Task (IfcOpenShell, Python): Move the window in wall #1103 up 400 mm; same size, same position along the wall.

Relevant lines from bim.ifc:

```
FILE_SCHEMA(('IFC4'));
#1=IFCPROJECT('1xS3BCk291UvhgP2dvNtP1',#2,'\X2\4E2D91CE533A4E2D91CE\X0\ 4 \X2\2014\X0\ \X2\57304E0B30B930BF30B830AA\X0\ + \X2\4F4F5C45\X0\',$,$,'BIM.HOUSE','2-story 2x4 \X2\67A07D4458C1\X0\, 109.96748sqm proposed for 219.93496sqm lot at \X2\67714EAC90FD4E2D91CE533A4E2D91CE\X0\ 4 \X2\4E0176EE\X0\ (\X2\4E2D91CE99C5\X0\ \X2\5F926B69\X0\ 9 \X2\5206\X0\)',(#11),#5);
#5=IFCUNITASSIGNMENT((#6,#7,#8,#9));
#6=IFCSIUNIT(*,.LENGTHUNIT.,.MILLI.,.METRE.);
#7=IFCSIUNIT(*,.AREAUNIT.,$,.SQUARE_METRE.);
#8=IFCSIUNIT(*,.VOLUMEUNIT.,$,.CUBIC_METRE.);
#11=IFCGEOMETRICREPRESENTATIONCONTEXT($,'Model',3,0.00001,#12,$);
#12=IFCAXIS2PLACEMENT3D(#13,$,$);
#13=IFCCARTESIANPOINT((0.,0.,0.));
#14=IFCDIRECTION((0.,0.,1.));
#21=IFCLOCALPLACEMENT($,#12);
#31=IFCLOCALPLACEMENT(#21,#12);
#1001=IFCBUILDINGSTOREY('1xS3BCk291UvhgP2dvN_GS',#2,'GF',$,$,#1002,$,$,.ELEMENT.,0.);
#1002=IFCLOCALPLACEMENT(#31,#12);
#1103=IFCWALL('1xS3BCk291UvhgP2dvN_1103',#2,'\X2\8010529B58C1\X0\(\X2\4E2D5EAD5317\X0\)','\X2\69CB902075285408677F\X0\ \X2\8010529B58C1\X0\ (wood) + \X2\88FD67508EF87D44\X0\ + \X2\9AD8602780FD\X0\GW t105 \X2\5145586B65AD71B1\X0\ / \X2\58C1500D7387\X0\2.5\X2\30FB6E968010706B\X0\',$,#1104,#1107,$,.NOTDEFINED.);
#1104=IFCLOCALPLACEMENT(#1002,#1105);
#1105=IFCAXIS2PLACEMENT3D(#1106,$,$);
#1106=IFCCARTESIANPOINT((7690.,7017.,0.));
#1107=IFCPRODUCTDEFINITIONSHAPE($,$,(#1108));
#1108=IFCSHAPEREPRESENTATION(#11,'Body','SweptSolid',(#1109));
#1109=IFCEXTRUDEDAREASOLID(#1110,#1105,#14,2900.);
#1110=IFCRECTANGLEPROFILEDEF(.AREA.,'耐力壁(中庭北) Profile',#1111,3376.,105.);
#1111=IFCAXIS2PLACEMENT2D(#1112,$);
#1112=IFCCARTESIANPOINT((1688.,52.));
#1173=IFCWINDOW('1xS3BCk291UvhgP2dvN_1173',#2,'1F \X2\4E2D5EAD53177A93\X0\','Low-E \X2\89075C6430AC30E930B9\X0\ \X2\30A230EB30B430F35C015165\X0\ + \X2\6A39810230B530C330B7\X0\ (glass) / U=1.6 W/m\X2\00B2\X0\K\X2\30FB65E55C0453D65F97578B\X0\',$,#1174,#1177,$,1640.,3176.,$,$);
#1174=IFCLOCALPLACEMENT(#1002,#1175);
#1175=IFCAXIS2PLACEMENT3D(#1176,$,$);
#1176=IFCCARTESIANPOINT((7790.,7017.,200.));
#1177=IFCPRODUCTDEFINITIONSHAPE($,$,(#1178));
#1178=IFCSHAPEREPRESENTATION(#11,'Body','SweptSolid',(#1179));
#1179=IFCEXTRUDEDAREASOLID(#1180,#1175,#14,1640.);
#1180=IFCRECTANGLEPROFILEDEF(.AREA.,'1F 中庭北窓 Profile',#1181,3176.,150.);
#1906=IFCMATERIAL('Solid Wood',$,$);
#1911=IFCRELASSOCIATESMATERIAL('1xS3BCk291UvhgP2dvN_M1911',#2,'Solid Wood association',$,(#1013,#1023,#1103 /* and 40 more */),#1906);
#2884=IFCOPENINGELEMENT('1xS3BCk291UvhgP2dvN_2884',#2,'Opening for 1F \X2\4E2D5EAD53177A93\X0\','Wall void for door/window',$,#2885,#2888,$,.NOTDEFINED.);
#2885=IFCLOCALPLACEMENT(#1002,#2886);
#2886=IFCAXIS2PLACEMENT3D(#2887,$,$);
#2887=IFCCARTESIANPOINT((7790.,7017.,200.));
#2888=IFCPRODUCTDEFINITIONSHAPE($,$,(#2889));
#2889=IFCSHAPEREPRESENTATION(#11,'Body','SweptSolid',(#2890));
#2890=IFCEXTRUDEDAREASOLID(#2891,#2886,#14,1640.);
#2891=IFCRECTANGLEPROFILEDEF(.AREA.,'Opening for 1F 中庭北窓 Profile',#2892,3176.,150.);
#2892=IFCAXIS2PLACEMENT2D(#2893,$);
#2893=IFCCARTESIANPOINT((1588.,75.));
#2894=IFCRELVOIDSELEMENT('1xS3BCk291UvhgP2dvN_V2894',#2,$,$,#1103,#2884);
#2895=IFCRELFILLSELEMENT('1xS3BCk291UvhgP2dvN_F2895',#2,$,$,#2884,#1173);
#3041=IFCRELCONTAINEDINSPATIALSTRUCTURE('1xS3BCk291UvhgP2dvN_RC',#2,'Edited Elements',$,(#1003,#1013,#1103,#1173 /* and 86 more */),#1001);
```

```python
import numpy as np
import ifcopenshell
import ifcopenshell.api.geometry
import ifcopenshell.util.placement
import ifcopenshell.util.unit

model = ifcopenshell.open("bim.ifc")
unit_scale = ifcopenshell.util.unit.calculate_unit_scale(model)

window = model.by_id(1173)
opening = window.FillsVoids[0].RelatingOpeningElement
dz = 0.4 / unit_scale

shift = np.array([0.0, 0.0, dz])
# The window is not placed relative to its opening, so move both.
for product in (opening, window):
    matrix = ifcopenshell.util.placement.get_local_placement(product.ObjectPlacement)
    matrix[:3, 3] += shift
    ifcopenshell.api.geometry.edit_object_placement(model, product=product, matrix=matrix, is_si=False)

print(f"moved by {dz * unit_scale:+.3f} m")

model.write("bim_edited.ifc")
```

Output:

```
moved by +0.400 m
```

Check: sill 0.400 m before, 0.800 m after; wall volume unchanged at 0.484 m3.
